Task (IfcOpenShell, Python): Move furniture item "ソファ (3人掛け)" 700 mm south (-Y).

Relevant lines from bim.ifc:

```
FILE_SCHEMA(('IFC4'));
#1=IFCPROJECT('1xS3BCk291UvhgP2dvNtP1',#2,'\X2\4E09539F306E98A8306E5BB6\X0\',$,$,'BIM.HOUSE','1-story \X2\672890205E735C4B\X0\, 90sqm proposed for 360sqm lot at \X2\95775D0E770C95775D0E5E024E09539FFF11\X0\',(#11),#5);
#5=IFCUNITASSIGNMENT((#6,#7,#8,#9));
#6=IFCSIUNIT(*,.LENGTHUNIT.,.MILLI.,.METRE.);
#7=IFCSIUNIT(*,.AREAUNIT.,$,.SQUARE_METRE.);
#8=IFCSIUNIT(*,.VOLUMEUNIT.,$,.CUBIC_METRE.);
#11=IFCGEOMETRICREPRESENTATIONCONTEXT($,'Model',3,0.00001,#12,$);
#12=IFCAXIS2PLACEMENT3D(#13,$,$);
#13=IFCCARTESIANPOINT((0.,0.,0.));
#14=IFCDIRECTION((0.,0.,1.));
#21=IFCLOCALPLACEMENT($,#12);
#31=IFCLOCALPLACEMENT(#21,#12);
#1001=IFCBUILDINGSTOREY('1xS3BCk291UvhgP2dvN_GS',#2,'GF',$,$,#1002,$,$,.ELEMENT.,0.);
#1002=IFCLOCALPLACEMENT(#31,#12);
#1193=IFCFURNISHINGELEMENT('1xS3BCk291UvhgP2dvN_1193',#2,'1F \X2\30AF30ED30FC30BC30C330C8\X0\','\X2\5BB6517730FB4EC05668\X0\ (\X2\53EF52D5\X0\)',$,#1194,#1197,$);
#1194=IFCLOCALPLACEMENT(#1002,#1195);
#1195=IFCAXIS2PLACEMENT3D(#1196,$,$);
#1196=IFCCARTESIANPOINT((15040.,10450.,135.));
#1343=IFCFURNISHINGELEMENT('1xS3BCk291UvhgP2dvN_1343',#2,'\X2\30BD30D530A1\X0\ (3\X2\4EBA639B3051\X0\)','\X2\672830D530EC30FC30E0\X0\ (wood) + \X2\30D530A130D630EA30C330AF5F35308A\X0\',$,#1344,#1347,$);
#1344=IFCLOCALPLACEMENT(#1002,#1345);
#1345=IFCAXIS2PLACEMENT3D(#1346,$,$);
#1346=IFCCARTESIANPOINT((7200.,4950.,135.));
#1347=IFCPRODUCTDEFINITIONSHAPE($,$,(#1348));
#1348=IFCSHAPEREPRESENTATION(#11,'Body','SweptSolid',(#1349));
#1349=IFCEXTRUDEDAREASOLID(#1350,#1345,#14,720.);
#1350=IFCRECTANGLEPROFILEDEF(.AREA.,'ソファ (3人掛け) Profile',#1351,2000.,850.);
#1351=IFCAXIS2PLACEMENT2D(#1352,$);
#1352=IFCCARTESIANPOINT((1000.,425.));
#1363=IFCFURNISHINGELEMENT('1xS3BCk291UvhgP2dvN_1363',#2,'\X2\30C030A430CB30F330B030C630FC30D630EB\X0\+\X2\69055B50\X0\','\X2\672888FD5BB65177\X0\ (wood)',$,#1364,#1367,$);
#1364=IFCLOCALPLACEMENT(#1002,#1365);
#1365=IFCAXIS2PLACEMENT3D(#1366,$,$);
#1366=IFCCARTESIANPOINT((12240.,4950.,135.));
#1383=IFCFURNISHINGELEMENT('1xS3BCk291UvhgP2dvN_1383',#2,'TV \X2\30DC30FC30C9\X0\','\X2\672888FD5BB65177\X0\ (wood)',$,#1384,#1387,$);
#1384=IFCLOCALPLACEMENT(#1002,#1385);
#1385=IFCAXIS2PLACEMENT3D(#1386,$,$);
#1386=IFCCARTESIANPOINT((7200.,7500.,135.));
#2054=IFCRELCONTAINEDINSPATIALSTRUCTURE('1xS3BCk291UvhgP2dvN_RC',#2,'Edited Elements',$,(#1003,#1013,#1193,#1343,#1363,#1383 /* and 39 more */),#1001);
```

```python
import ifcopenshell
import ifcopenshell.api.geometry
import ifcopenshell.util.placement

model = ifcopenshell.open("bim.ifc")

item = model.by_id(1343)
matrix = ifcopenshell.util.placement.get_local_placement(item.ObjectPlacement)
matrix[1, 3] -= 700.0
ifcopenshell.api.geometry.edit_object_placement(model, product=item, matrix=matrix, is_si=False)

print(ifcopenshell.util.placement.get_local_placement(item.ObjectPlacement).round(3) + 0.0)

model.write("bim_v2.ifc")
```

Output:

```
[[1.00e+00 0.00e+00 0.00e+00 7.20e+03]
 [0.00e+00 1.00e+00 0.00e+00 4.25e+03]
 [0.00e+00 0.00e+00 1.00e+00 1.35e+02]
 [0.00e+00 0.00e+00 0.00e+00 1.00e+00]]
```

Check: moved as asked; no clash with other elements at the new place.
